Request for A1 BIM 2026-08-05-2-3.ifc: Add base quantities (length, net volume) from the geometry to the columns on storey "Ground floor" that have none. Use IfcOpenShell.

First a look at what the model holds.

```python
import ifcopenshell
import ifcopenshell.util.element
import ifcopenshell.util.unit

model = ifcopenshell.open("A1 BIM 2026-08-05-2-3.ifc")
print(model.schema)
for unit_type in ("LENGTHUNIT", "AREAUNIT", "VOLUMEUNIT"):
    print(unit_type, ifcopenshell.util.unit.calculate_unit_scale(model, unit_type))
storey = next(s for s in model.by_type("IfcBuildingStorey") if s.Name == "Ground floor")
columns = [e for e in ifcopenshell.util.element.get_decomposition(storey) if e.is_a("IfcColumn")]
for e in sorted(columns, key=lambda e: e.id()):
    print(e.id(), e.is_a(), e.Name, list(ifcopenshell.util.element.get_psets(e, qtos_only=True)), sep=" | ")
```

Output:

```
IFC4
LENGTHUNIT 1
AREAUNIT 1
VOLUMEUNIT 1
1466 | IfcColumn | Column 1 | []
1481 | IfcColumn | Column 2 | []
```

```python
import ifcopenshell
import ifcopenshell.api.pset
import ifcopenshell.geom
import ifcopenshell.util.element
import ifcopenshell.util.shape
import ifcopenshell.util.unit

model = ifcopenshell.open("A1 BIM 2026-08-05-2-3.ifc")
unit_scale = ifcopenshell.util.unit.calculate_unit_scale(model)
volume_scale = ifcopenshell.util.unit.calculate_unit_scale(model, "VOLUMEUNIT")
settings = ifcopenshell.geom.settings()

storey = next(s for s in model.by_type("IfcBuildingStorey") if s.Name == "Ground floor")
columns = [e for e in ifcopenshell.util.element.get_decomposition(storey) if e.is_a("IfcColumn")]

for e in sorted(columns, key=lambda e: e.id()):
    if ifcopenshell.util.element.get_psets(e, qtos_only=True, should_inherit=False):
        continue
    # Geometry comes back in metres, in the element's own axes.
    shape = ifcopenshell.geom.create_shape(settings, e)
    values = {
        "Length": ifcopenshell.util.shape.get_z(shape.geometry) / unit_scale,
        "NetVolume": ifcopenshell.util.shape.get_volume(shape.geometry) / volume_scale,
    }
    qto = ifcopenshell.api.pset.add_qto(model, product=e, name="Qto_ColumnBaseQuantities")
    ifcopenshell.api.pset.edit_qto(model, qto=qto, properties=values)
    print(e.id(), {k: round(v, 3) for k, v in values.items()})

model.write("A1 BIM 2026-08-05-2-3_rev.ifc")
```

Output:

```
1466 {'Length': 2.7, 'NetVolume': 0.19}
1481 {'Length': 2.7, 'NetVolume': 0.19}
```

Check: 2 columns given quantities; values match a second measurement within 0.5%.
